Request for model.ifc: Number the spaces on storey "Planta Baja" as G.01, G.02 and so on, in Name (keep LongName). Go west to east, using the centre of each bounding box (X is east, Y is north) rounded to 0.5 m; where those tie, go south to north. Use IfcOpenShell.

First a look at what the model holds.

```python
import ifcopenshell
import ifcopenshell.util.element
import ifcopenshell.util.placement

model = ifcopenshell.open("model.ifc")
print(model.schema)
storey = next(s for s in model.by_type("IfcBuildingStorey") if s.Name == "Planta Baja")
spaces = [e for e in ifcopenshell.util.element.get_decomposition(storey) if e.is_a("IfcSpace")]
for e in sorted(spaces, key=lambda e: e.id()):
    origin = ifcopenshell.util.placement.get_local_placement(e.ObjectPlacement)[:3, 3]
    print(e.id(), e.Name, e.LongName, origin.round(2) + 0.0, sep=" | ")
```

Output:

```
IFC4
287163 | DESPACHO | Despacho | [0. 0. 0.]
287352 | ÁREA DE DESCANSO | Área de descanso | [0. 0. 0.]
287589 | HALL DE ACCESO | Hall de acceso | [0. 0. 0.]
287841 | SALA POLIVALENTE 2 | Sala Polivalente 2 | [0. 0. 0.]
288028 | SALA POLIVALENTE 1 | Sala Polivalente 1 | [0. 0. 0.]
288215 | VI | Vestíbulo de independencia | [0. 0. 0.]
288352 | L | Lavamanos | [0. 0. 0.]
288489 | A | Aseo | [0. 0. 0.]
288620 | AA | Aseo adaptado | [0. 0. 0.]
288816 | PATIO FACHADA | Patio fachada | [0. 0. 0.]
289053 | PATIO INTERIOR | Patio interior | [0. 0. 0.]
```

```python
import ifcopenshell
import ifcopenshell.geom
import ifcopenshell.util.element
import ifcopenshell.util.shape

model = ifcopenshell.open("model.ifc")
settings = ifcopenshell.geom.settings()
settings.set("use-world-coords", True)


def centre(element):
    shape = ifcopenshell.geom.create_shape(settings, element)
    return ifcopenshell.util.shape.get_bbox_centroid(shape.geometry)


storey = next(s for s in model.by_type("IfcBuildingStorey") if s.Name == "Planta Baja")
spaces = [e for e in ifcopenshell.util.element.get_decomposition(storey) if e.is_a("IfcSpace")]

# Insertion points can sit at a corner or the storey origin, so sort by the geometry (in metres).
centres = {e: centre(e) for e in spaces}
spaces.sort(key=lambda e: (round(centres[e][0] / 0.5), centres[e][1]))

for i, e in enumerate(spaces, start=1):
    number = f"G.{i:02d}"
    e.Name = number
    print(e.id(), number)

model.write("model_updated.ifc")
```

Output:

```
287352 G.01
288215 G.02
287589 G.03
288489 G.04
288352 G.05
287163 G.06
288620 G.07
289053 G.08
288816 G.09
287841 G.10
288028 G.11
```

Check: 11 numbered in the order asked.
